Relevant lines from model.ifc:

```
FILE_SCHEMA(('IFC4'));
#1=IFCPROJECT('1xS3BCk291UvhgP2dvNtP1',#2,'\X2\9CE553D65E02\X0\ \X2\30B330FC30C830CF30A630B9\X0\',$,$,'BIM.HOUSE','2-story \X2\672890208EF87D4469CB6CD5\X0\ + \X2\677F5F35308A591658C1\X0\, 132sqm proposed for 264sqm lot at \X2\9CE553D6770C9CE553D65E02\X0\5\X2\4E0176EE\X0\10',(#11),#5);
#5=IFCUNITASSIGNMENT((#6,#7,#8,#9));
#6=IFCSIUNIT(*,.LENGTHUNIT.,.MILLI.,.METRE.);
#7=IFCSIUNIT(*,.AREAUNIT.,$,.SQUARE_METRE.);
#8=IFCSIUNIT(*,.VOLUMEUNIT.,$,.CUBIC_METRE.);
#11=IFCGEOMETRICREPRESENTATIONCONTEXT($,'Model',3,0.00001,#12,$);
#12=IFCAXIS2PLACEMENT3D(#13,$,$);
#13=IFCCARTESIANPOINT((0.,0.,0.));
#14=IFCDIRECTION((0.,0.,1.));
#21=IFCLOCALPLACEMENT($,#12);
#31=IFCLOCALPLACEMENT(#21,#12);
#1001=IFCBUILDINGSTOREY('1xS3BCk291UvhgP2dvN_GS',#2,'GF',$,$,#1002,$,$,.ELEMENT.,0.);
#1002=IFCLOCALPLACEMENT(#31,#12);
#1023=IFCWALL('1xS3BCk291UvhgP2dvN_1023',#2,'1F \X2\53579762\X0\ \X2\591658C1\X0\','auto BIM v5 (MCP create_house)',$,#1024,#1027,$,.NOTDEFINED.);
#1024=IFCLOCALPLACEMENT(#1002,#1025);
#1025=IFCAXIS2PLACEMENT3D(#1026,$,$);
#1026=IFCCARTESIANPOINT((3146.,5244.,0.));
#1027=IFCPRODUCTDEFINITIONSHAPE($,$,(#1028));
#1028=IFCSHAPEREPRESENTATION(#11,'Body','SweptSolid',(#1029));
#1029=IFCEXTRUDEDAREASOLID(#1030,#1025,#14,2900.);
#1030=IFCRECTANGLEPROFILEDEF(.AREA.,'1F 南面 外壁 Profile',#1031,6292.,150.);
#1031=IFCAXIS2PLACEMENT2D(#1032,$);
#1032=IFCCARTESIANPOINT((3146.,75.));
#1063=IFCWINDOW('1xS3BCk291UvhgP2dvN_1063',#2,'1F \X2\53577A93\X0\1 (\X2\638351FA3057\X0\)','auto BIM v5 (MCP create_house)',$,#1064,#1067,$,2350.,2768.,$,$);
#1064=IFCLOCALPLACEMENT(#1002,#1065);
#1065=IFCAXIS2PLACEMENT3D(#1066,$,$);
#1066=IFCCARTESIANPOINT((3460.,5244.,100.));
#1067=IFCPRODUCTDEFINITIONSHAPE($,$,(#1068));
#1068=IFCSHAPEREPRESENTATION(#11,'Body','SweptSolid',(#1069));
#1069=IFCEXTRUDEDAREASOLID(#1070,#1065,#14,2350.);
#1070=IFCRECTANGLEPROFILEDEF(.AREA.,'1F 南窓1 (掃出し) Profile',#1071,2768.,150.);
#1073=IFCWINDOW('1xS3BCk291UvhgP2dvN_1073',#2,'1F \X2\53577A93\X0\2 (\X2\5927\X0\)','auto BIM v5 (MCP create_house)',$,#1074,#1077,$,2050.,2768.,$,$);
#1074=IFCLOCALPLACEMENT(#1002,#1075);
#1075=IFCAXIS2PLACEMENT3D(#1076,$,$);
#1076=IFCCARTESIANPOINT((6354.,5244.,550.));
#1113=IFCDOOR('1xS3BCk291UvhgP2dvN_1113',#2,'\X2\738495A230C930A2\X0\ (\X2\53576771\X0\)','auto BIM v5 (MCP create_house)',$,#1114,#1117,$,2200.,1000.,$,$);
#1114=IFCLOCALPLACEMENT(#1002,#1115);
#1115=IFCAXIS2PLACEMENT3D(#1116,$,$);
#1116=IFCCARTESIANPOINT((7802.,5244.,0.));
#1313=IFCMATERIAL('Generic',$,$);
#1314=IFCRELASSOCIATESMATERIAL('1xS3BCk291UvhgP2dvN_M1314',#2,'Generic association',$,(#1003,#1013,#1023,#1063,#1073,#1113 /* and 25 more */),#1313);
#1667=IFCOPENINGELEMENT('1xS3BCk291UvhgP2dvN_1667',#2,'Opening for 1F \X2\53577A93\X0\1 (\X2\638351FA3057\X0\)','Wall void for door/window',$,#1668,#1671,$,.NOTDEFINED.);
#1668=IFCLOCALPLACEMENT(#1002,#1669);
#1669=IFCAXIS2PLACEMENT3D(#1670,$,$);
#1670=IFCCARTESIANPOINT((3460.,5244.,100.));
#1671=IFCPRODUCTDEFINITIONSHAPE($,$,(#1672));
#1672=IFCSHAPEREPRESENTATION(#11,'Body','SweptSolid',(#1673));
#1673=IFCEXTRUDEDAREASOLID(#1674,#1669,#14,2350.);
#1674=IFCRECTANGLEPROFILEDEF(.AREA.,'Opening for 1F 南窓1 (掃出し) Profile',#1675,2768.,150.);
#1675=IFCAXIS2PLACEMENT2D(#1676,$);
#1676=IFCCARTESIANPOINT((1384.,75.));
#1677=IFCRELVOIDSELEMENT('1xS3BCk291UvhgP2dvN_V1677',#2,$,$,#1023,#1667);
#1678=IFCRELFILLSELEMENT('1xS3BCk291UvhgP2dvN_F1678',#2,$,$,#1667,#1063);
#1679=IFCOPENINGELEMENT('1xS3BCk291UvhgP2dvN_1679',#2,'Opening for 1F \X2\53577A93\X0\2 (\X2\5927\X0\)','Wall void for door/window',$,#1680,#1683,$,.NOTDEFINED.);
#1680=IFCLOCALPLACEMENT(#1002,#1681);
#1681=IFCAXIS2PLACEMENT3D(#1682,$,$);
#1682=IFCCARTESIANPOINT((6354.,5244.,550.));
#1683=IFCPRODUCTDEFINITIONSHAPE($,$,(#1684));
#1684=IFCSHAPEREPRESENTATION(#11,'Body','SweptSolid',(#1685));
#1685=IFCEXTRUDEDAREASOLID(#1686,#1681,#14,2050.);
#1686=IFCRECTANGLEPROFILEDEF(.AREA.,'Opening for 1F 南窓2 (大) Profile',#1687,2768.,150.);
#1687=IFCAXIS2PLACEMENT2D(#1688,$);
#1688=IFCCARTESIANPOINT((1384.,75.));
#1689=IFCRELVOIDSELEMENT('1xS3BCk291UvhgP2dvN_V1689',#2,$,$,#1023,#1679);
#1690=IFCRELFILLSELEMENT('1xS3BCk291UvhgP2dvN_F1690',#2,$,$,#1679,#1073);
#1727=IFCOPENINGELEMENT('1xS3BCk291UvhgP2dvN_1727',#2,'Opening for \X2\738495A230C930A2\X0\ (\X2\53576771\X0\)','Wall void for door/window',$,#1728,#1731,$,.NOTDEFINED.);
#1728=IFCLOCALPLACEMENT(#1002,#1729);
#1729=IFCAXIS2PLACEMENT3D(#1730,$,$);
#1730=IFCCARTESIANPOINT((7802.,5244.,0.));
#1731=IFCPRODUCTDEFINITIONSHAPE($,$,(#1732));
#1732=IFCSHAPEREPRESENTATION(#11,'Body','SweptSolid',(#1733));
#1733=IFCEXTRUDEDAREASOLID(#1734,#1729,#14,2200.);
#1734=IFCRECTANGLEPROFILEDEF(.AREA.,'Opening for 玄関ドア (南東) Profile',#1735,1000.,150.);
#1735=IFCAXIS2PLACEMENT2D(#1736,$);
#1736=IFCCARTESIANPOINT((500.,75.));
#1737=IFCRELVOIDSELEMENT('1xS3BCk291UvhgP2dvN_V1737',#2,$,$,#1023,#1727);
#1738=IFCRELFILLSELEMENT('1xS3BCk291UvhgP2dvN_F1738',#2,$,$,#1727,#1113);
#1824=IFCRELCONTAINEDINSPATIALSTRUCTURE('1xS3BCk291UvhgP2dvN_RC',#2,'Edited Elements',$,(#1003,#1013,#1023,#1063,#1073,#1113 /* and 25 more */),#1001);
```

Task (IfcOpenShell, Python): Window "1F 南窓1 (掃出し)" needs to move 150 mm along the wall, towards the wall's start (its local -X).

```python
import ifcopenshell
import ifcopenshell.api.geometry
import ifcopenshell.util.placement
import ifcopenshell.util.unit

model = ifcopenshell.open("model.ifc")
unit_scale = ifcopenshell.util.unit.calculate_unit_scale(model)

window = model.by_guid("1xS3BCk291UvhgP2dvN_1063")
opening = window.FillsVoids[0].RelatingOpeningElement
wall = opening.VoidsElements[0].RelatingBuildingElement

wall_matrix = ifcopenshell.util.placement.get_local_placement(wall.ObjectPlacement)
shift = wall_matrix[:3, 0] * -0.15 / unit_scale
before = ifcopenshell.util.placement.get_local_placement(window.ObjectPlacement)[:3, 3].copy()

# The window is not placed relative to its opening, so move both.
for product in (opening, window):
    matrix = ifcopenshell.util.placement.get_local_placement(product.ObjectPlacement)
    matrix[:3, 3] += shift
    ifcopenshell.api.geometry.edit_object_placement(model, product=product, matrix=matrix, is_si=False)

after = ifcopenshell.util.placement.get_local_placement(window.ObjectPlacement)[:3, 3]
print("window moved by", (after - before).round(3) + 0.0)

model.write("model-out.ifc")
```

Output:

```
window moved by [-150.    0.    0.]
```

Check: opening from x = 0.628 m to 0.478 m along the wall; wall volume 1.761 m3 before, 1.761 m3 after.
